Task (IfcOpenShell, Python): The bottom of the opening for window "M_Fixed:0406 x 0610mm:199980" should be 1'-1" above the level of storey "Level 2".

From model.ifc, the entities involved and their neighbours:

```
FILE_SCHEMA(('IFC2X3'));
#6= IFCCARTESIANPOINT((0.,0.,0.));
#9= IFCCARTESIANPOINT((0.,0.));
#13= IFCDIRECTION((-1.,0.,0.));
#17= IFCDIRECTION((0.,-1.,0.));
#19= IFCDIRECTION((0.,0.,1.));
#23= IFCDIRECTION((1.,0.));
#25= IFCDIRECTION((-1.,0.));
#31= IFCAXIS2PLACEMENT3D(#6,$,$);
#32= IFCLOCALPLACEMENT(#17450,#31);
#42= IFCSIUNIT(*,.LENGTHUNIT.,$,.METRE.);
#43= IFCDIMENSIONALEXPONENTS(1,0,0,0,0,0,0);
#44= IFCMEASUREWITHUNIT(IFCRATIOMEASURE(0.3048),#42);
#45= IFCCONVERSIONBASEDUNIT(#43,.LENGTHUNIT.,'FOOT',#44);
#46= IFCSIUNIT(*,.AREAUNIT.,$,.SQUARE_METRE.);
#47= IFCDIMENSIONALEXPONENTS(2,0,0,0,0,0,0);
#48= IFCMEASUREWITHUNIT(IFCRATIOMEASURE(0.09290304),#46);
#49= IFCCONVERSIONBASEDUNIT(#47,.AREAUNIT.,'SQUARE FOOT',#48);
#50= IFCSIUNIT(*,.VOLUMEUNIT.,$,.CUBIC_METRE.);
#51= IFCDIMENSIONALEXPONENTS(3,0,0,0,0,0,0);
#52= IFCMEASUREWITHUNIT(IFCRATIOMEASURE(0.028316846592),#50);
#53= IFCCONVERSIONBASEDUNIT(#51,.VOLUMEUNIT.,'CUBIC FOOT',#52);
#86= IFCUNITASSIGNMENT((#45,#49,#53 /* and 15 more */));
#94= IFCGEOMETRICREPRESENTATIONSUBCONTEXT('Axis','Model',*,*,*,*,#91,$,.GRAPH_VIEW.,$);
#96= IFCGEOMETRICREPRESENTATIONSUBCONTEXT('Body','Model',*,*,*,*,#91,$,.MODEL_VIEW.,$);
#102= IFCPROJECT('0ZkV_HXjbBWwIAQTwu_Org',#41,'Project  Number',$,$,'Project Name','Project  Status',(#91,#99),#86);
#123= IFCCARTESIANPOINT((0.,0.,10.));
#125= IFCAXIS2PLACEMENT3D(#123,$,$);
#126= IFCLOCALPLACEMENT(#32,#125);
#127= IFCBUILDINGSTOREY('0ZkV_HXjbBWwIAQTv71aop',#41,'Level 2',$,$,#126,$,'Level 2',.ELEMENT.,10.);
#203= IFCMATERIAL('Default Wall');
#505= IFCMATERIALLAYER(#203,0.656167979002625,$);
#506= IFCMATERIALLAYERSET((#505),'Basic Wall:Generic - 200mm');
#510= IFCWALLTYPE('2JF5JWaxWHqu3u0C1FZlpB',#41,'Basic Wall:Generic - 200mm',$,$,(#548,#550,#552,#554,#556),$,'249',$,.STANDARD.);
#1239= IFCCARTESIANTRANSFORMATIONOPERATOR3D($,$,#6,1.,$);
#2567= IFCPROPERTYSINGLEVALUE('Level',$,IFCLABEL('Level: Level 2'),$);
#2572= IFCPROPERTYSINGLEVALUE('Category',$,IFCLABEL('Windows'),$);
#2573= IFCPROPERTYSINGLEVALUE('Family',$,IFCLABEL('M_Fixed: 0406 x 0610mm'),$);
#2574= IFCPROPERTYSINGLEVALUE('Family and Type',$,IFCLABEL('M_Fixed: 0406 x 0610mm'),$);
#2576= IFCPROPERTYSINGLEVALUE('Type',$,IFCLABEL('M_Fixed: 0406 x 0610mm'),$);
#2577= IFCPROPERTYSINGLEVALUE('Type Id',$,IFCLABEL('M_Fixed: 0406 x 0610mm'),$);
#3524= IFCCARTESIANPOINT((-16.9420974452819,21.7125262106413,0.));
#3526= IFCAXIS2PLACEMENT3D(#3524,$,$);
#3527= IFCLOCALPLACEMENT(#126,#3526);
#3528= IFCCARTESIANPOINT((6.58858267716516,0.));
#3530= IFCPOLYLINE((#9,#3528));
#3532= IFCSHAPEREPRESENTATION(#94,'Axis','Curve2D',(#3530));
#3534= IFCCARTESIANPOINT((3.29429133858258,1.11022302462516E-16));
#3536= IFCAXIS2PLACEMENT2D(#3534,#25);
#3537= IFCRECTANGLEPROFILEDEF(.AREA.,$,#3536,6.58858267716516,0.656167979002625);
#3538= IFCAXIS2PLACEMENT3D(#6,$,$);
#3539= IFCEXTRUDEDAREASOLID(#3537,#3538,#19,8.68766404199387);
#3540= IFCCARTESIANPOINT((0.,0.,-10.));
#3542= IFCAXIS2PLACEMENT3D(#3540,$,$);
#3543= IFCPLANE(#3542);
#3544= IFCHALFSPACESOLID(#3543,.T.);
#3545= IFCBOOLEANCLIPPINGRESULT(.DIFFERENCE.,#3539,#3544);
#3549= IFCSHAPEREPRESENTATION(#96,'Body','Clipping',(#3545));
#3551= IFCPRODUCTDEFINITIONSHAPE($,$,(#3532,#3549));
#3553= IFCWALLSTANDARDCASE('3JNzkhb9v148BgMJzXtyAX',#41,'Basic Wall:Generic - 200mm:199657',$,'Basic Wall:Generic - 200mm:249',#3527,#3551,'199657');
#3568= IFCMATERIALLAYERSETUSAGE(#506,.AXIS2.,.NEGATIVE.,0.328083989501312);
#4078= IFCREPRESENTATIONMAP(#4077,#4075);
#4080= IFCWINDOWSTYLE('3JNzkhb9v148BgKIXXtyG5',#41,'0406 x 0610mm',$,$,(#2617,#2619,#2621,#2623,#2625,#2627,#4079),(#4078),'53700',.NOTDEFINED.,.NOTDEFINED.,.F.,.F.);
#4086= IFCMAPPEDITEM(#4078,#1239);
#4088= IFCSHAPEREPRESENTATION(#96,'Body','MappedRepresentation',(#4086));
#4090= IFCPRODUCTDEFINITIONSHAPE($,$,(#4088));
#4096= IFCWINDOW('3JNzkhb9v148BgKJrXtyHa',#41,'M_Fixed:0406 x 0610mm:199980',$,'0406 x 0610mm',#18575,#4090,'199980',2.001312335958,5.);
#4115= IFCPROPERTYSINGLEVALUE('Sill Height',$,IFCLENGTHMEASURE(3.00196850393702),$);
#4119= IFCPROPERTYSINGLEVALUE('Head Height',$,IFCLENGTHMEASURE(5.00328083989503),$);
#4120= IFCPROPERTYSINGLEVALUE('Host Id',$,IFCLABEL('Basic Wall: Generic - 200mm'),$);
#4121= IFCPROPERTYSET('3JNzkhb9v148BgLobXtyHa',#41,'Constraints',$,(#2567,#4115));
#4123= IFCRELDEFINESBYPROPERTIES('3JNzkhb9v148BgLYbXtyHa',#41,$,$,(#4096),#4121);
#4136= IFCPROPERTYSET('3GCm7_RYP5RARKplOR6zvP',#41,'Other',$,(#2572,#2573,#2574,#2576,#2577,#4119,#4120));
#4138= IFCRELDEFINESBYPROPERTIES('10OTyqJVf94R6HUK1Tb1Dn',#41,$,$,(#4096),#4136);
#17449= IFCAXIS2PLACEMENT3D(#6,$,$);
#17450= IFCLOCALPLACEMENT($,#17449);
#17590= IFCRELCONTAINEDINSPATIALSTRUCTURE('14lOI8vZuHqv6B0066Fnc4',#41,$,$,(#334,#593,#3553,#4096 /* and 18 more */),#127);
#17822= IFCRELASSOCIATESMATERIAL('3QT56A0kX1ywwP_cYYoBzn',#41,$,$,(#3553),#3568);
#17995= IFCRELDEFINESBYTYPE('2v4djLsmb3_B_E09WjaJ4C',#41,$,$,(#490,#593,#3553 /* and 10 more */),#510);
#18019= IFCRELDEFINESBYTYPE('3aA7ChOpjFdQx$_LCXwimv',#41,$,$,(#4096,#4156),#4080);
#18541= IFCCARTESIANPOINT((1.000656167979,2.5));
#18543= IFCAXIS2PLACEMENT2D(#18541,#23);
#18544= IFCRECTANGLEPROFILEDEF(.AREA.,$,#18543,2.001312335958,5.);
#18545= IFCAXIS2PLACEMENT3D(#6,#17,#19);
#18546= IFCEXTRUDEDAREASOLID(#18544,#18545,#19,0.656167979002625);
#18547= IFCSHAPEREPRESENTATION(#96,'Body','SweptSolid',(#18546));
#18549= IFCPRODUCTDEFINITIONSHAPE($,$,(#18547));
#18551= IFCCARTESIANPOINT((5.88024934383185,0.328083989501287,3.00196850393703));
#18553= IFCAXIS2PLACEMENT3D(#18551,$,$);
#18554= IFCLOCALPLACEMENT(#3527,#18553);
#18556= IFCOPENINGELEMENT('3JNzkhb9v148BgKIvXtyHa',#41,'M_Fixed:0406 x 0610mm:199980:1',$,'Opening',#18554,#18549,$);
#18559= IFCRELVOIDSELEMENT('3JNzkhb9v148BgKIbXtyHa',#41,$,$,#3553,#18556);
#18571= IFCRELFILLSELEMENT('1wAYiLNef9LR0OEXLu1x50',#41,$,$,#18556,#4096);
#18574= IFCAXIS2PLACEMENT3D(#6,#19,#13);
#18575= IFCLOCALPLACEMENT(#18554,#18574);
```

```python
import numpy as np
import ifcopenshell
import ifcopenshell.api.geometry
import ifcopenshell.api.pset
import ifcopenshell.geom
import ifcopenshell.util.element
import ifcopenshell.util.placement
import ifcopenshell.util.shape
import ifcopenshell.util.unit

model = ifcopenshell.open("model.ifc")
unit_scale = ifcopenshell.util.unit.calculate_unit_scale(model)

window = model.by_guid("3JNzkhb9v148BgKJrXtyHa")
opening = window.FillsVoids[0].RelatingOpeningElement
storey = ifcopenshell.util.element.get_container(window, ifc_class="IfcBuildingStorey")
level = ifcopenshell.util.placement.get_local_placement(storey.ObjectPlacement)[2, 3]

# The opening's origin need not be at the sill, so measure its lowest point.
shape = ifcopenshell.geom.create_shape(ifcopenshell.geom.settings(), opening)
bottom = ifcopenshell.util.shape.get_shape_bottom_elevation(shape, shape.geometry) / unit_scale
dz = level + 13 * 0.0254 / unit_scale - bottom

shift = np.array([0.0, 0.0, dz])
# The window is placed relative to its opening, so it follows when the opening moves.
matrix = ifcopenshell.util.placement.get_local_placement(opening.ObjectPlacement)
matrix[:3, 3] += shift
ifcopenshell.api.geometry.edit_object_placement(
    model, product=opening, matrix=matrix, is_si=False, should_transform_children=True
)

# Keep the stored heights in step.
pset = model.by_id(ifcopenshell.util.element.get_pset(window, "Constraints", should_inherit=False)["id"])
ifcopenshell.api.pset.edit_pset(model, pset=pset, properties={
    "Sill Height": model.create_entity("IfcLengthMeasure", ifcopenshell.util.element.get_pset(window, "Constraints", "Sill Height") + dz),
})
pset = model.by_id(ifcopenshell.util.element.get_pset(window, "Other", should_inherit=False)["id"])
ifcopenshell.api.pset.edit_pset(model, pset=pset, properties={
    "Head Height": model.create_entity("IfcLengthMeasure", ifcopenshell.util.element.get_pset(window, "Other", "Head Height") + dz),
})

print(f"moved by {dz * unit_scale:+.3f} m")

model.write("model_edited.ifc")
```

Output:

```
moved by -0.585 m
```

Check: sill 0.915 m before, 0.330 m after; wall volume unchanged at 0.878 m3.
